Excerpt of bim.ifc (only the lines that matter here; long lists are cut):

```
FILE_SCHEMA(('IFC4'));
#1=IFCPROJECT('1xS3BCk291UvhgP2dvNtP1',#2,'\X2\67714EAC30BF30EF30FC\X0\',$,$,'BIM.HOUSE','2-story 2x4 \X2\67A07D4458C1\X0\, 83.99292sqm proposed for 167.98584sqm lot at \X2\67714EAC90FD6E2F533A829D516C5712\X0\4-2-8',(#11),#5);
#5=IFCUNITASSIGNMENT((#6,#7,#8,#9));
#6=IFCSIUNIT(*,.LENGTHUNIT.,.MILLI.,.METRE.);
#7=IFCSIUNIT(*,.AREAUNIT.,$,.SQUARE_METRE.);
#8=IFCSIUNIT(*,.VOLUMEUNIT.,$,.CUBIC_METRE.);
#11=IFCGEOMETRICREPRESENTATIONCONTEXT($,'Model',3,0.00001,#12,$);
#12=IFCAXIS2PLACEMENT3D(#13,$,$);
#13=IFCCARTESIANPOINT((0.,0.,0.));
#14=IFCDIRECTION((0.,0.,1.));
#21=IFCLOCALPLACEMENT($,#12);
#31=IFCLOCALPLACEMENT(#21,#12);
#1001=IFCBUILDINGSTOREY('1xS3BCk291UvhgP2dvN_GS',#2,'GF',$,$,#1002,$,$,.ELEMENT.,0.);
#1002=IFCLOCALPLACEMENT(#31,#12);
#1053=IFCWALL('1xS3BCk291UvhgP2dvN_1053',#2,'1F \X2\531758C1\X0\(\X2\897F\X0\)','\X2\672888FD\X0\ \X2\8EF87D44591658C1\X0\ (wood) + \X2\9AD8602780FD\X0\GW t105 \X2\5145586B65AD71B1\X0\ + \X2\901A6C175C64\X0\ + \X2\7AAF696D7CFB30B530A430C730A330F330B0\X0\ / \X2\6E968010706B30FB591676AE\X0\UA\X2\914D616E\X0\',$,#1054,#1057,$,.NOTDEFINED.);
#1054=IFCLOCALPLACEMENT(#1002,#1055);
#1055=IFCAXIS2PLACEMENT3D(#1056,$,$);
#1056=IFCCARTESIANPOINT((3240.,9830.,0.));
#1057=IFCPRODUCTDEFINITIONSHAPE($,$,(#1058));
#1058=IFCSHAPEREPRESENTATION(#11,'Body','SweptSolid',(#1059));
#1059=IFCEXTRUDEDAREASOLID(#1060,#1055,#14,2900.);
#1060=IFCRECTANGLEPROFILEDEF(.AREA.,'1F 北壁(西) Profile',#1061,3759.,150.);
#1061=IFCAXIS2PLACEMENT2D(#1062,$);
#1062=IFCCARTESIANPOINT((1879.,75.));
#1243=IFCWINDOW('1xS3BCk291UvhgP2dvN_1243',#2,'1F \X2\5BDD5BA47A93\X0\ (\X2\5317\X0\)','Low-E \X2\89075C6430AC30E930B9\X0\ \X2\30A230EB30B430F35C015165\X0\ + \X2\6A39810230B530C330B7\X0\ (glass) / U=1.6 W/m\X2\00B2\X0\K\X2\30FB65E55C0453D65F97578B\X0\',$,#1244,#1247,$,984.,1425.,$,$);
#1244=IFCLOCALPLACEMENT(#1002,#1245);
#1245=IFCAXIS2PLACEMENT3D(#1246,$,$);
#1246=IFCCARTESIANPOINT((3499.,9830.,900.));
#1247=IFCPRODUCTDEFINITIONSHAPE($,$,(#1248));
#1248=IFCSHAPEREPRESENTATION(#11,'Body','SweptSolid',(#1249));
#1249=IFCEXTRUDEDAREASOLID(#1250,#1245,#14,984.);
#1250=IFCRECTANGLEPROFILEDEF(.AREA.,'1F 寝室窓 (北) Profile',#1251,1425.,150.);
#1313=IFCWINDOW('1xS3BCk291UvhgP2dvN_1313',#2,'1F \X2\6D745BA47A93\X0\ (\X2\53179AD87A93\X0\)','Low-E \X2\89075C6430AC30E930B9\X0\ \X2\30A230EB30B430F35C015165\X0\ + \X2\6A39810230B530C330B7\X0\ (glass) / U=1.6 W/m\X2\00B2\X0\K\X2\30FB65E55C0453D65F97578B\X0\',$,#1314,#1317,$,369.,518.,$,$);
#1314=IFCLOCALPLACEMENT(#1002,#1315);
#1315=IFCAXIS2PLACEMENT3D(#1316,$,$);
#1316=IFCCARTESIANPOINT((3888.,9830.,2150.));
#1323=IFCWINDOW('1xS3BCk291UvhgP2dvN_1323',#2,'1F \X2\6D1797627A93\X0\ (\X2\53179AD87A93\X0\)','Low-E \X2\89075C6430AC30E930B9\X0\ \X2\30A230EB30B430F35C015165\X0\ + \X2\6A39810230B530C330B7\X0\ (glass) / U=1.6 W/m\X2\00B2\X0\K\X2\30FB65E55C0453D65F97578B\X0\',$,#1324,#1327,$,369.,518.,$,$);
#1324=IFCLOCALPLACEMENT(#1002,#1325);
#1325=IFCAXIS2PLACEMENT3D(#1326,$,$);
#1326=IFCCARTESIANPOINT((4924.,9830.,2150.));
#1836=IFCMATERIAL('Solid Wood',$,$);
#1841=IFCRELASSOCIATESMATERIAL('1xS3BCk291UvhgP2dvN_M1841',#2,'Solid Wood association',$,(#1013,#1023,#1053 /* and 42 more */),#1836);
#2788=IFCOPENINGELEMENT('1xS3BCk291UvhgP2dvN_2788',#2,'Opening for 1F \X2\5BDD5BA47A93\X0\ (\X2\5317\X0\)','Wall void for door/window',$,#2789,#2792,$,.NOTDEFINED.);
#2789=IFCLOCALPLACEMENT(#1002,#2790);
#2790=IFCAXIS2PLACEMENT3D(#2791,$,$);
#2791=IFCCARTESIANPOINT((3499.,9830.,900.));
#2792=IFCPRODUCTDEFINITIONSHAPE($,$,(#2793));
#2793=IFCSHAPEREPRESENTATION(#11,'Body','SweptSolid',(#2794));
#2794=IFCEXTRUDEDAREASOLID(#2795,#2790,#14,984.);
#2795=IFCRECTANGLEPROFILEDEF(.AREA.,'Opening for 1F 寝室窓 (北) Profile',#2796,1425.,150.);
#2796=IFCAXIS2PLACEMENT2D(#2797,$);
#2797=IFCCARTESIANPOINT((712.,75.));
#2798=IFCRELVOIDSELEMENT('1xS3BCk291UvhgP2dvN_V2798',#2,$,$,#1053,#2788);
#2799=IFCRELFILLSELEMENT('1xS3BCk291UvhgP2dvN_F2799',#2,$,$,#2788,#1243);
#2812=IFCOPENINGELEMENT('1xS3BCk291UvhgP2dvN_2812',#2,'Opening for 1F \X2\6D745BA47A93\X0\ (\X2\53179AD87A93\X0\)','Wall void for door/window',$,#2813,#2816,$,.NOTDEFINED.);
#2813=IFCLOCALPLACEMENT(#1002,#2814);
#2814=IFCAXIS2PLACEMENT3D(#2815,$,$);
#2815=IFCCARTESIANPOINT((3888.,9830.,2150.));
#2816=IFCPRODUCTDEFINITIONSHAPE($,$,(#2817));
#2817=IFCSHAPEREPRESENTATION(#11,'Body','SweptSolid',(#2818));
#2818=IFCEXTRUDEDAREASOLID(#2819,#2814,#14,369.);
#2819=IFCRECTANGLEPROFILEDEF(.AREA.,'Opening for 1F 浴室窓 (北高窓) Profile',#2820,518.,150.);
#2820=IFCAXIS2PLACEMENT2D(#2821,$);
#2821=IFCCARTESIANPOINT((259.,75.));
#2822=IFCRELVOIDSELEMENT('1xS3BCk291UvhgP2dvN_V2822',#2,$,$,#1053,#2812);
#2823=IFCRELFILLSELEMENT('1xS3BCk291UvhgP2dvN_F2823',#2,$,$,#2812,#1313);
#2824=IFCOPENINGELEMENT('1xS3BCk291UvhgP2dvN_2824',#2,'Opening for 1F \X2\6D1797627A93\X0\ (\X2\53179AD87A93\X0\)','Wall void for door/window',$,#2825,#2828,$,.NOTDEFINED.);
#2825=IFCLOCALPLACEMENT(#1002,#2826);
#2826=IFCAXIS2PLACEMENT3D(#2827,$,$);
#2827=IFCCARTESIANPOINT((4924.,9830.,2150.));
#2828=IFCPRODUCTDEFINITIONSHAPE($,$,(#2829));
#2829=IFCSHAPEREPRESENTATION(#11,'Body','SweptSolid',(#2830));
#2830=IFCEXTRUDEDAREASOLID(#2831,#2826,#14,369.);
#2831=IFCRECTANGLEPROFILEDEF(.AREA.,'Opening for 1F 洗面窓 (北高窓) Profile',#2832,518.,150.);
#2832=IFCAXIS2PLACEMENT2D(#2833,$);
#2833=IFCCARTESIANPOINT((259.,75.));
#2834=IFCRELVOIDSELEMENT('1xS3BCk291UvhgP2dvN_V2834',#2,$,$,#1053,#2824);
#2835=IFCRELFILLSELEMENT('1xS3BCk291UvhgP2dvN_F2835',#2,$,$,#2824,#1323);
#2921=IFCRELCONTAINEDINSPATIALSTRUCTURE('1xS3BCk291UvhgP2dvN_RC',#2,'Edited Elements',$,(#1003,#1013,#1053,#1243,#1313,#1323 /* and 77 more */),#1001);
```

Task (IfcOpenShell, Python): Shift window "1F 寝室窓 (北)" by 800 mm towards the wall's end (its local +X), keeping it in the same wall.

```python
import ifcopenshell
import ifcopenshell.api.geometry
import ifcopenshell.util.placement
import ifcopenshell.util.unit

model = ifcopenshell.open("bim.ifc")
unit_scale = ifcopenshell.util.unit.calculate_unit_scale(model)

window = model.by_id(1243)
opening = window.FillsVoids[0].RelatingOpeningElement
wall = opening.VoidsElements[0].RelatingBuildingElement

wall_matrix = ifcopenshell.util.placement.get_local_placement(wall.ObjectPlacement)
shift = wall_matrix[:3, 0] * 0.8 / unit_scale
before = ifcopenshell.util.placement.get_local_placement(window.ObjectPlacement)[:3, 3].copy()

# The window is not placed relative to its opening, so move both.
for product in (opening, window):
    matrix = ifcopenshell.util.placement.get_local_placement(product.ObjectPlacement)
    matrix[:3, 3] += shift
    ifcopenshell.api.geometry.edit_object_placement(model, product=product, matrix=matrix, is_si=False)

after = ifcopenshell.util.placement.get_local_placement(window.ObjectPlacement)[:3, 3]
print("window moved by", (after - before).round(3) + 0.0)

model.write("bim_edited.ifc")
```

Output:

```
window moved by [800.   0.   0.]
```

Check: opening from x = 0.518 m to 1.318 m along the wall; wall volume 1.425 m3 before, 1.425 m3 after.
